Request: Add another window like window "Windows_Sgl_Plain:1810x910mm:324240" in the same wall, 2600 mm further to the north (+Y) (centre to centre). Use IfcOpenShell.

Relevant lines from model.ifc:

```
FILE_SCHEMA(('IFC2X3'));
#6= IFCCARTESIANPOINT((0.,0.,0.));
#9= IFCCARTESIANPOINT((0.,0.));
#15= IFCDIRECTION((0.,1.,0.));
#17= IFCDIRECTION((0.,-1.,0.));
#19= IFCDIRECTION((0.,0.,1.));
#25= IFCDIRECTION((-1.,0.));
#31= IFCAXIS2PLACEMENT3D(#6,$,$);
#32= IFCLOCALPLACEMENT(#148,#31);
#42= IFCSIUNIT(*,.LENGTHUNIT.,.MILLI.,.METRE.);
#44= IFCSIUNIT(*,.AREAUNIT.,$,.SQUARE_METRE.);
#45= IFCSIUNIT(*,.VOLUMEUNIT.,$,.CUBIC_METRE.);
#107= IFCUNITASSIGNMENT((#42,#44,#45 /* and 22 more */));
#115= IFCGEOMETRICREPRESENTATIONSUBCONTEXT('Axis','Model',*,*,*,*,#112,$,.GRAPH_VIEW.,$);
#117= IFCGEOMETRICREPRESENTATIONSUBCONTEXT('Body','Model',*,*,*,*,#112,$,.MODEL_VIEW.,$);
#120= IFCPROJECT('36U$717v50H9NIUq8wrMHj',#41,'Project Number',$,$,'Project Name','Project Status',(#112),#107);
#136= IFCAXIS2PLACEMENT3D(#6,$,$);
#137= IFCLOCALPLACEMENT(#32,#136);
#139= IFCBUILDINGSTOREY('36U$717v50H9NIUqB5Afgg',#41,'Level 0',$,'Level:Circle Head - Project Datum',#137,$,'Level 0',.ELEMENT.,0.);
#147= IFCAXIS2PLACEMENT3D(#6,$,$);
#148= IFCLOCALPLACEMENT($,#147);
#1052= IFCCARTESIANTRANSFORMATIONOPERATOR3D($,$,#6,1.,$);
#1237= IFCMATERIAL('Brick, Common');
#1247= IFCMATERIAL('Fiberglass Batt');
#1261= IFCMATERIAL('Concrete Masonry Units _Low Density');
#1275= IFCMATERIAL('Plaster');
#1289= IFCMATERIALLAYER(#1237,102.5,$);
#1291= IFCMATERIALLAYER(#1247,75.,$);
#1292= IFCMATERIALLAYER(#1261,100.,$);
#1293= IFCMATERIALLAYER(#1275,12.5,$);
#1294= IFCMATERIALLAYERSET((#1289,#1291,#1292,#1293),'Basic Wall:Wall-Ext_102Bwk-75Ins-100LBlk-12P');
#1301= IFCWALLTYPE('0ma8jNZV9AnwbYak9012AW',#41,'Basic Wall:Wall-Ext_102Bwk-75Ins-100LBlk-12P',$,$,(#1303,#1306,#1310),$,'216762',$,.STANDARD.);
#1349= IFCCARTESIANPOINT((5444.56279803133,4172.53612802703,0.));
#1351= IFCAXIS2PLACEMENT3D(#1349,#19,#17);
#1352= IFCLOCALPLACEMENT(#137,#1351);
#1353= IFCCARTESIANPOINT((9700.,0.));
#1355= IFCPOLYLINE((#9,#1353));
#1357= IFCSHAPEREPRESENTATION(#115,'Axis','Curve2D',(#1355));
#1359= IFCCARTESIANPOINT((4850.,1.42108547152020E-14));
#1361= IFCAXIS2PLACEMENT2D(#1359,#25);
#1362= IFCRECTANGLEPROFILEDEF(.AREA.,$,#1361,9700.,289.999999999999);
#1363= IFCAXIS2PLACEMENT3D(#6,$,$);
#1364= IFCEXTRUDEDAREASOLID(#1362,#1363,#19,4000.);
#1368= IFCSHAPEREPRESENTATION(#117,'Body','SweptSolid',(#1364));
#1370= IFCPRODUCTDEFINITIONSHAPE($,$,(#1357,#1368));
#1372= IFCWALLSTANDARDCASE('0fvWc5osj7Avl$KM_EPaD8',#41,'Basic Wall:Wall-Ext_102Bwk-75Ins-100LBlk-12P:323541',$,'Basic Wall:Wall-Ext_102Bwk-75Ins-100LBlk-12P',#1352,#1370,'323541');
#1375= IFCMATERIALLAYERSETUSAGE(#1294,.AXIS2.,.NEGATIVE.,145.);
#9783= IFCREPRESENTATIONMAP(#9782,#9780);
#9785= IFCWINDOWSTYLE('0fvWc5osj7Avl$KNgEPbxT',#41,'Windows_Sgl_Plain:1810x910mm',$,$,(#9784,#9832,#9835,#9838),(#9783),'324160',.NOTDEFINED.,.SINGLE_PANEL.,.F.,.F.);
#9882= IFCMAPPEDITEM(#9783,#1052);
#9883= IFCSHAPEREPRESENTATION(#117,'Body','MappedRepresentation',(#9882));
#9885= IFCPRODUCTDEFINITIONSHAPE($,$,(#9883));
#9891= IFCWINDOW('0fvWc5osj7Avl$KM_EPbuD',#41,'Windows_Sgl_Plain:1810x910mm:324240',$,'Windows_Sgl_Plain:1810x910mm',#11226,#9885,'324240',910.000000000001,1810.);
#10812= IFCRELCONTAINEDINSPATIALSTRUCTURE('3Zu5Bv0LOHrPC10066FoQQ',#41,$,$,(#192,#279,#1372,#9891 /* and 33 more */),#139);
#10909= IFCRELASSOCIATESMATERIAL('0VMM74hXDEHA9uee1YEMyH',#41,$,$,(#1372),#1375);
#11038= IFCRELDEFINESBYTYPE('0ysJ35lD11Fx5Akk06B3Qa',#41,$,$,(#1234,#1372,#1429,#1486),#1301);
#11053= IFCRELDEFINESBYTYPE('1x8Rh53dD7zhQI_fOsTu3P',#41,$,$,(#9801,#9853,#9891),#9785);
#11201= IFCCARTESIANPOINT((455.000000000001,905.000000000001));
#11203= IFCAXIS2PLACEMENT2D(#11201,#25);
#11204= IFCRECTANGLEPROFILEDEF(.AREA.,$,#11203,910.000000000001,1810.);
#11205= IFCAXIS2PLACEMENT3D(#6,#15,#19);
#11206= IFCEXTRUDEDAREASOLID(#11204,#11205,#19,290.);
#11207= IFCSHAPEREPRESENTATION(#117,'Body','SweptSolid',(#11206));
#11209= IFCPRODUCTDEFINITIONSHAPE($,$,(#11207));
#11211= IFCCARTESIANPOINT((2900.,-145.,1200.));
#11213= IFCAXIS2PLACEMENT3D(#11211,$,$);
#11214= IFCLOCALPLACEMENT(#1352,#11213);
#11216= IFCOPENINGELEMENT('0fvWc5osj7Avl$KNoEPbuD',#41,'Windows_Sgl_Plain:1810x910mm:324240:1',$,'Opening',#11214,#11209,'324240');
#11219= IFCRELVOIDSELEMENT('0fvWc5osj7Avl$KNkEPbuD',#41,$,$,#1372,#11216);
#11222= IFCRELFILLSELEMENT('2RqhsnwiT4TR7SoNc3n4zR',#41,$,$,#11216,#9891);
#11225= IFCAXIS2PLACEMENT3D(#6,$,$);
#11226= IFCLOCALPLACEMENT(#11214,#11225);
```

```python
import ifcopenshell
import ifcopenshell.api.feature
import ifcopenshell.api.geometry
import ifcopenshell.api.root
import ifcopenshell.geom
import ifcopenshell.util.element
import ifcopenshell.util.placement
import ifcopenshell.util.shape

model = ifcopenshell.open("model.ifc")
settings = ifcopenshell.geom.settings()


def volume(element):
    """Net volume in cubic metres, openings subtracted."""
    shape = ifcopenshell.geom.create_shape(settings, element)
    return ifcopenshell.util.shape.get_volume(shape.geometry)


def reuse_history(source, copy):
    """copy_class also copies each property set's owner history, people and application; keep the originals."""
    for rel in copy.IsDefinedBy:
        if rel.is_a("IfcRelDefinesByProperties") and (history := rel.RelatingPropertyDefinition.OwnerHistory):
            rel.RelatingPropertyDefinition.OwnerHistory = source.OwnerHistory
            ifcopenshell.util.element.remove_deep2(model, history)


window = model.by_id(9891)
opening = window.FillsVoids[0].RelatingOpeningElement
wall = opening.VoidsElements[0].RelatingBuildingElement
before = volume(wall)
shift = ifcopenshell.util.placement.get_local_placement(wall.ObjectPlacement)[:3, 0] * -2600.0

# copy_class copies the void relationship, type, container and properties, but no geometry.
new_opening = ifcopenshell.api.root.copy_class(model, product=opening)
new_opening.Representation = ifcopenshell.util.element.copy_deep(
    model, opening.Representation, exclude=["IfcGeometricRepresentationContext", "IfcRepresentationMap"]
)
new_opening.Name = "Windows_Sgl_Plain:1810x910mm"
new_opening.Tag = None
new_window = ifcopenshell.api.root.copy_class(model, product=window)
new_window.Representation = ifcopenshell.util.element.copy_deep(
    model, window.Representation, exclude=["IfcGeometricRepresentationContext", "IfcRepresentationMap"]
)
new_window.Name = "Windows_Sgl_Plain:1810x910mm"
new_window.Tag = None
reuse_history(window, new_window)
fills = ifcopenshell.api.feature.add_filling(model, opening=new_opening, element=new_window)
fills.OwnerHistory = new_window.OwnerHistory  # required in IFC2X3

for old, new in ((opening, new_opening), (window, new_window)):
    matrix = ifcopenshell.util.placement.get_local_placement(old.ObjectPlacement)
    matrix[:3, 3] += shift
    ifcopenshell.api.geometry.edit_object_placement(model, product=new, matrix=matrix, is_si=False)

after = volume(wall)

print(f"wall volume {before:.3f} -> {after:.3f} m3")

model.write("model_updated.ifc")
```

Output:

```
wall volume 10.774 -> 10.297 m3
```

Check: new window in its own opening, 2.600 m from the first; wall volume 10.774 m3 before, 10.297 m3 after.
